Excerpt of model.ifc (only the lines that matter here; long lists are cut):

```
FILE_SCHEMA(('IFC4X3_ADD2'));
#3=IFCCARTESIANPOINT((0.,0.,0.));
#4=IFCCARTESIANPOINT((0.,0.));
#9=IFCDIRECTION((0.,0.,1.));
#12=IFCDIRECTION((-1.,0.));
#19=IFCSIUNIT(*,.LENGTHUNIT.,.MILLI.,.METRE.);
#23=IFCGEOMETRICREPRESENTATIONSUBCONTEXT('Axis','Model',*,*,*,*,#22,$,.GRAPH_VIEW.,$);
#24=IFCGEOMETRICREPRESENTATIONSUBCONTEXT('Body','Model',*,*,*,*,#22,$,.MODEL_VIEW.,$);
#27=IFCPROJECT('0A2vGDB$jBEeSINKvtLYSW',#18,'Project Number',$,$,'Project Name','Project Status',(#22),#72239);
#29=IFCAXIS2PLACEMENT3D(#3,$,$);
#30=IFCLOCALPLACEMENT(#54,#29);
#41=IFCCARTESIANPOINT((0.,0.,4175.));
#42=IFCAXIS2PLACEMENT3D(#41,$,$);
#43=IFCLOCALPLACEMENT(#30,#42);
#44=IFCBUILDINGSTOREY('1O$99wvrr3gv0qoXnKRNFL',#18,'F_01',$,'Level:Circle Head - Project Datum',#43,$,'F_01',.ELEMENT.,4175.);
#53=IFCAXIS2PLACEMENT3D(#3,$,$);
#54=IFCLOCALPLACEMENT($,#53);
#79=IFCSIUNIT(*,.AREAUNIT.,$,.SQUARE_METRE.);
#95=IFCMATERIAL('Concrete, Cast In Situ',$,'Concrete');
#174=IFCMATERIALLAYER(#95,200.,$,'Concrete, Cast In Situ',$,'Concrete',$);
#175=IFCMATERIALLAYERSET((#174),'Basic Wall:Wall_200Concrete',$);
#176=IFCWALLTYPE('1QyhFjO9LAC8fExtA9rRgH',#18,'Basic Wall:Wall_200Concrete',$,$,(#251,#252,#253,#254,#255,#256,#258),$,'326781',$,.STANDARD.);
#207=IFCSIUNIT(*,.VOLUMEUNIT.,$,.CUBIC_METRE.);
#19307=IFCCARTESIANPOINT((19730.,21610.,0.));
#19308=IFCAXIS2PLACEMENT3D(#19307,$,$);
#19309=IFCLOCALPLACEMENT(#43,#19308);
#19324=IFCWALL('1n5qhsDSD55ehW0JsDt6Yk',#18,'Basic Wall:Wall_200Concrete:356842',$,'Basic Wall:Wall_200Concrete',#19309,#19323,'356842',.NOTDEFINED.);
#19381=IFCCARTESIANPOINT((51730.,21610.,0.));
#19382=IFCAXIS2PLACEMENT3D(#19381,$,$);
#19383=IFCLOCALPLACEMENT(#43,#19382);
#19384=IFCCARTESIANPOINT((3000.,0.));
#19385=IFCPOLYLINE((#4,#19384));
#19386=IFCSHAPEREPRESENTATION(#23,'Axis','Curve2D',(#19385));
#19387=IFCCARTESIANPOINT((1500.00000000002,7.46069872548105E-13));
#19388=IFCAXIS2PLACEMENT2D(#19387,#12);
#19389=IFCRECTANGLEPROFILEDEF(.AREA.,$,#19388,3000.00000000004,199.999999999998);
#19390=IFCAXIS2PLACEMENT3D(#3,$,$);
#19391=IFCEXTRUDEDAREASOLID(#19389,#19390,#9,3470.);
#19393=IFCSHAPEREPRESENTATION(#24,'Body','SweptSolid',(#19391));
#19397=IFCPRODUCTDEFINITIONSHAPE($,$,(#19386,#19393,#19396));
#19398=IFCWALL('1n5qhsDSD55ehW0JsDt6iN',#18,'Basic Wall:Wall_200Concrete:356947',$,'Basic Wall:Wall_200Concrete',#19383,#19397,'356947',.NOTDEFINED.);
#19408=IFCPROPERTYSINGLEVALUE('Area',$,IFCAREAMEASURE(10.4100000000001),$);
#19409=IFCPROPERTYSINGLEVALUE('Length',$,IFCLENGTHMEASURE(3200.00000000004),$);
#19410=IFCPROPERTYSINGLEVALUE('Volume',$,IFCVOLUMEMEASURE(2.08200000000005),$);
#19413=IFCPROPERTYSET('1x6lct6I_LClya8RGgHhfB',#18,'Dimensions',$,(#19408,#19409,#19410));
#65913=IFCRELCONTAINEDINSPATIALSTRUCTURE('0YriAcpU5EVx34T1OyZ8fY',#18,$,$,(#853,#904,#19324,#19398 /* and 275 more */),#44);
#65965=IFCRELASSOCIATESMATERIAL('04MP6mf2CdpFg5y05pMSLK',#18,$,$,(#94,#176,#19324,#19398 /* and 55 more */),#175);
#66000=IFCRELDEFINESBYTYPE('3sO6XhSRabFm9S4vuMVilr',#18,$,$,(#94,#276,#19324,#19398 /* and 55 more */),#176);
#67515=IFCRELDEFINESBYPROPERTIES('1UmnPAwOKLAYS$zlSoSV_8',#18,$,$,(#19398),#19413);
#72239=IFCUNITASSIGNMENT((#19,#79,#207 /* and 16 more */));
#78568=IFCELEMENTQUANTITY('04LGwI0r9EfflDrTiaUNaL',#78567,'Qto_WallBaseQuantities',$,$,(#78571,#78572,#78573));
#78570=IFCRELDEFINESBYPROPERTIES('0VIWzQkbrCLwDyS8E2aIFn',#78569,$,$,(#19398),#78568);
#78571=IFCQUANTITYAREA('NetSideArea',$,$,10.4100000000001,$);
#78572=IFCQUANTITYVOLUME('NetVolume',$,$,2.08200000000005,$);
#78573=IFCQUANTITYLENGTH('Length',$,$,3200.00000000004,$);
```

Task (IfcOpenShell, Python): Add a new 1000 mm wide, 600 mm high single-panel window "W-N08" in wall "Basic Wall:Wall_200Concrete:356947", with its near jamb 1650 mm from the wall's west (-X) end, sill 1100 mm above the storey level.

```python
import numpy as np
import ifcopenshell
import ifcopenshell.api.feature
import ifcopenshell.api.geometry
import ifcopenshell.api.pset
import ifcopenshell.api.root
import ifcopenshell.api.spatial
import ifcopenshell.geom
import ifcopenshell.util.element
import ifcopenshell.util.placement
import ifcopenshell.util.representation
import ifcopenshell.util.shape
import ifcopenshell.util.unit

model = ifcopenshell.open("model.ifc")
unit_scale = ifcopenshell.util.unit.calculate_unit_scale(model)
area_scale = ifcopenshell.util.unit.calculate_unit_scale(model, "AREAUNIT")
volume_scale = ifcopenshell.util.unit.calculate_unit_scale(model, "VOLUMEUNIT")
settings = ifcopenshell.geom.settings()


def volume(element):
    """Net volume in cubic metres, openings subtracted."""
    shape = ifcopenshell.geom.create_shape(settings, element)
    return ifcopenshell.util.shape.get_volume(shape.geometry)


wall = model.by_guid("1n5qhsDSD55ehW0JsDt6iN")
storey = ifcopenshell.util.element.get_container(wall, ifc_class="IfcBuildingStorey")
context = ifcopenshell.util.representation.get_context(model, "Model", "Body", "MODEL_VIEW")
before = volume(wall)

width, height, from_end, sill = 1, 0.6, 1.65, 1.1  # metres

# The wall runs along its own X axis, and the end named is its -X end.
wall_shape = ifcopenshell.geom.create_shape(settings, wall)
x, y, z = ifcopenshell.util.shape.get_vertices(wall_shape.geometry).T
start = x.min() + from_end
face, thickness = float(y.min()), float(y.max() - y.min())
wall_matrix = ifcopenshell.util.placement.get_local_placement(wall.ObjectPlacement)
level = ifcopenshell.util.placement.get_local_placement(storey.ObjectPlacement)[2, 3]


def in_wall(x, y):
    """Placement at x, y metres in the wall's axes, at sill height."""
    matrix = wall_matrix.copy()
    matrix[:, 3] = wall_matrix @ np.array([x / unit_scale, y / unit_scale, 0.0, 1.0])
    matrix[2, 3] = level + sill / unit_scale
    return matrix


# Opening: a box that overshoots both wall faces by 50 mm.
opening = ifcopenshell.api.root.create_entity(model, ifc_class="IfcOpeningElement", predefined_type="OPENING")
box = ifcopenshell.api.geometry.add_wall_representation(
    model, context=context, length=width, height=height, thickness=thickness + 0.1
)
ifcopenshell.api.geometry.assign_representation(model, product=opening, representation=box)
ifcopenshell.api.geometry.edit_object_placement(model, product=opening, matrix=in_wall(start, face - 0.05), is_si=False)
ifcopenshell.api.feature.add_feature(model, feature=opening, element=wall)

window = ifcopenshell.api.root.create_entity(model, ifc_class="IfcWindow", name="W-N08", predefined_type="WINDOW")
window.OverallWidth, window.OverallHeight = width / unit_scale, height / unit_scale
window.PartitioningType = "SINGLE_PANEL"
body = ifcopenshell.api.geometry.add_window_representation(
    model,
    context=context,
    overall_width=window.OverallWidth,
    overall_height=window.OverallHeight,
    partition_type="SINGLE_PANEL",
)
ifcopenshell.api.geometry.assign_representation(model, product=window, representation=body)
ifcopenshell.api.spatial.assign_container(model, products=[window], relating_structure=storey)
ifcopenshell.api.feature.add_filling(model, opening=opening, element=window)

# Centre the window in the wall's thickness.
ifcopenshell.api.geometry.edit_object_placement(model, product=window, matrix=in_wall(start, face), is_si=False)
window_shape = ifcopenshell.geom.create_shape(settings, window)
depth = ifcopenshell.util.shape.get_vertices(window_shape.geometry)[:, 1]
offset = face + thickness / 2 - (depth.min() + depth.max()) / 2
ifcopenshell.api.geometry.edit_object_placement(model, product=window, matrix=in_wall(start, offset), is_si=False)

after = volume(wall)

# Update the wall's stored quantities.
pset = model.by_id(ifcopenshell.util.element.get_pset(wall, "Dimensions", should_inherit=False)["id"])
ifcopenshell.api.pset.edit_pset(model, pset=pset, properties={
    "Area": model.create_entity("IfcAreaMeasure", after / thickness / area_scale),
    "Volume": model.create_entity("IfcVolumeMeasure", after / volume_scale),
})
qto = model.by_id(ifcopenshell.util.element.get_pset(wall, "Qto_WallBaseQuantities", should_inherit=False)["id"])
ifcopenshell.api.pset.edit_qto(model, qto=qto, properties={
    "NetSideArea": after / thickness / area_scale,
    "NetVolume": after / volume_scale,
})

print(f"wall volume {before:.3f} -> {after:.3f} m3")

model.write("model-out.ifc")
```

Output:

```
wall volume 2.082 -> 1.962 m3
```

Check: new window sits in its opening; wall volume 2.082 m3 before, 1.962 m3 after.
